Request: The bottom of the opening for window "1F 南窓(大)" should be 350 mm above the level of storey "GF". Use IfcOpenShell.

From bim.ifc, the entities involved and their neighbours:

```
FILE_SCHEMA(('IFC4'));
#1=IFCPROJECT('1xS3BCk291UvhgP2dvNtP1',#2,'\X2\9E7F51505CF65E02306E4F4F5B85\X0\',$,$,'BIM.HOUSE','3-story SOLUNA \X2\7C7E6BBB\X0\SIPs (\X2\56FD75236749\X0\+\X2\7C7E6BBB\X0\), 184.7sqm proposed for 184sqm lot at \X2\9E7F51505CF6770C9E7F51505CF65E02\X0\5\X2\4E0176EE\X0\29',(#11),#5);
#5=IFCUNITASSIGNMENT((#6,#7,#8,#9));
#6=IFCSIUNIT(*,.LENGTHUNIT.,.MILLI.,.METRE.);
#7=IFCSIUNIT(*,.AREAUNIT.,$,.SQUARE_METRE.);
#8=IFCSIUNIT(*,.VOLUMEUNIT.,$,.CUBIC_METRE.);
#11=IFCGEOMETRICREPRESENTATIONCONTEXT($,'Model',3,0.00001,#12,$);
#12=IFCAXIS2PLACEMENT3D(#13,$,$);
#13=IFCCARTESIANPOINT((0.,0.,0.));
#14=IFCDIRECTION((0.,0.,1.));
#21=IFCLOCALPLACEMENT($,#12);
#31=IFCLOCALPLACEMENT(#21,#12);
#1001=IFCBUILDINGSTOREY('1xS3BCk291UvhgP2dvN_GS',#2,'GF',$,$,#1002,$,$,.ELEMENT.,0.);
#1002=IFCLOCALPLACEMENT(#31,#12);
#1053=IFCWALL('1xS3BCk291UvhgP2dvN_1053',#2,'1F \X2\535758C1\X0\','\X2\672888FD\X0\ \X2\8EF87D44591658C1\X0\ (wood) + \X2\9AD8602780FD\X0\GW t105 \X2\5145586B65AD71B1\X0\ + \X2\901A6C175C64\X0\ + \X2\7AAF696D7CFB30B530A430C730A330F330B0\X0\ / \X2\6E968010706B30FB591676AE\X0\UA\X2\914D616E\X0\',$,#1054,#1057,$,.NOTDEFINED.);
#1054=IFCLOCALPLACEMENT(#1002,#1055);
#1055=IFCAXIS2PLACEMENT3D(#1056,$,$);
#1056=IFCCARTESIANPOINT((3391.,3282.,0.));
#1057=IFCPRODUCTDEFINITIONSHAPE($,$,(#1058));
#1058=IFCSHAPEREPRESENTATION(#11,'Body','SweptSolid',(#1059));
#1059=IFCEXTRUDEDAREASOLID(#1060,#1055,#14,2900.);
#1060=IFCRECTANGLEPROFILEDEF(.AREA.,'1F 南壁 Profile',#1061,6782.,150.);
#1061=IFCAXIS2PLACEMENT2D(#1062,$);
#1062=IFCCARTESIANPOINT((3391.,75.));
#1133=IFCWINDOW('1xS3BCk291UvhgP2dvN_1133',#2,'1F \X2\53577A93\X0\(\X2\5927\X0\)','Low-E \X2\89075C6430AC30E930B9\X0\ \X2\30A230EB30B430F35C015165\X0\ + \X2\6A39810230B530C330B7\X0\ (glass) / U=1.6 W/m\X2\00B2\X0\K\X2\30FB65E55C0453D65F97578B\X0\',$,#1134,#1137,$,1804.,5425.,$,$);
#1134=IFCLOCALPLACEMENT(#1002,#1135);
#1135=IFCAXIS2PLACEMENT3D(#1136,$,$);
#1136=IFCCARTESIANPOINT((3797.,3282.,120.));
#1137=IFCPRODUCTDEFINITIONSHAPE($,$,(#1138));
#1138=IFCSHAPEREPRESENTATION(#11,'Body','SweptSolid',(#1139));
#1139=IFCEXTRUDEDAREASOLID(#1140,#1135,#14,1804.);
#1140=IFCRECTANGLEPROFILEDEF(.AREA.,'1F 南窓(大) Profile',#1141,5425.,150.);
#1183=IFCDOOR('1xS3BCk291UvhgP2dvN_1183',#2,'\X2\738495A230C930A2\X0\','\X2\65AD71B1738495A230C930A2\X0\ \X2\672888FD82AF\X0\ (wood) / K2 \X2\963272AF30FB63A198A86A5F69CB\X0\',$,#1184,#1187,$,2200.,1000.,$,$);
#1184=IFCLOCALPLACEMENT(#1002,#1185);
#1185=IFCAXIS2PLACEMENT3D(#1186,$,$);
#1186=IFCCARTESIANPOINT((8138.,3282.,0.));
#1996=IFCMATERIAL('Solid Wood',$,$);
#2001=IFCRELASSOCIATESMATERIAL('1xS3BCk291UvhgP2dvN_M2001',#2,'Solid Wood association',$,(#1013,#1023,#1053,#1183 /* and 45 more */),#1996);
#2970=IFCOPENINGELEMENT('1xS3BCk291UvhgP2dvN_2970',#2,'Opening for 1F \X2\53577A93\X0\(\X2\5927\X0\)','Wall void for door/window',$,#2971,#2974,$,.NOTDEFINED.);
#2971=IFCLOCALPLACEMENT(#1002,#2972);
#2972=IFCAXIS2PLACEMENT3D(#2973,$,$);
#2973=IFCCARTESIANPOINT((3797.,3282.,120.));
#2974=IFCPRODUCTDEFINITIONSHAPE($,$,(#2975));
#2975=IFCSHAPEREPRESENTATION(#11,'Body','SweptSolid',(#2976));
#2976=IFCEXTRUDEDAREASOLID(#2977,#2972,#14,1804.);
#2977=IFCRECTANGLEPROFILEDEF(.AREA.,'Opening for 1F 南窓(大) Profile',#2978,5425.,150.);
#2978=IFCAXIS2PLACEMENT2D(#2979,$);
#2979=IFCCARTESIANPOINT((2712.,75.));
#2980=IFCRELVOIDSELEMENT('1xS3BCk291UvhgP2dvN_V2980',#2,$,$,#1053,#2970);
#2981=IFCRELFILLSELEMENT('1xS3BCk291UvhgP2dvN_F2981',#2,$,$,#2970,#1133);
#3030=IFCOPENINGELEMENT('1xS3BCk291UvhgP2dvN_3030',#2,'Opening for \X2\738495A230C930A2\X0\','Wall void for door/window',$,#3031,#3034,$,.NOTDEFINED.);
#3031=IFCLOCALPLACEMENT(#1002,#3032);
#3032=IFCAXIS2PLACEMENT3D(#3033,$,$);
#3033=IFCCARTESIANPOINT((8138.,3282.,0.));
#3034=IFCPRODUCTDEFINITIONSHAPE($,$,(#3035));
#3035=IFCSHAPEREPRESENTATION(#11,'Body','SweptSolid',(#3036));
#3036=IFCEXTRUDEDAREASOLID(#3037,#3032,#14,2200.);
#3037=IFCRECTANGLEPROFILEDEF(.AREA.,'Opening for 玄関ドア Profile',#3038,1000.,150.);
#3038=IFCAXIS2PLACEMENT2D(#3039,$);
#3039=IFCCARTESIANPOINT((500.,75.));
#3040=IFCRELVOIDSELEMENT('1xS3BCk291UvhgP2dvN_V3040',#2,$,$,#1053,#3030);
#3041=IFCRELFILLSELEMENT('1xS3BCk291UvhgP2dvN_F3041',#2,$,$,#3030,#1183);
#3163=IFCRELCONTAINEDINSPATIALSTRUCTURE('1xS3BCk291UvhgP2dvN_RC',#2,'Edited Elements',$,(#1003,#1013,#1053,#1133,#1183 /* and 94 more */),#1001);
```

```python
import numpy as np
import ifcopenshell
import ifcopenshell.api.geometry
import ifcopenshell.geom
import ifcopenshell.util.element
import ifcopenshell.util.placement
import ifcopenshell.util.shape
import ifcopenshell.util.unit

model = ifcopenshell.open("bim.ifc")
unit_scale = ifcopenshell.util.unit.calculate_unit_scale(model)

window = model.by_guid("1xS3BCk291UvhgP2dvN_1133")
opening = window.FillsVoids[0].RelatingOpeningElement
storey = ifcopenshell.util.element.get_container(window, ifc_class="IfcBuildingStorey")
level = ifcopenshell.util.placement.get_local_placement(storey.ObjectPlacement)[2, 3]

# The opening's origin need not be at the sill, so measure its lowest point.
shape = ifcopenshell.geom.create_shape(ifcopenshell.geom.settings(), opening)
bottom = ifcopenshell.util.shape.get_shape_bottom_elevation(shape, shape.geometry) / unit_scale
dz = level + 350.0 - bottom

shift = np.array([0.0, 0.0, dz])
# The window is not placed relative to its opening, so move both.
for product in (opening, window):
    matrix = ifcopenshell.util.placement.get_local_placement(product.ObjectPlacement)
    matrix[:3, 3] += shift
    ifcopenshell.api.geometry.edit_object_placement(model, product=product, matrix=matrix, is_si=False)

print(f"moved by {dz * unit_scale:+.3f} m")

model.write("bim_updated.ifc")
```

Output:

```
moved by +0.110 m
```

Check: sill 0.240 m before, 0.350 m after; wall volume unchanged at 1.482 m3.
